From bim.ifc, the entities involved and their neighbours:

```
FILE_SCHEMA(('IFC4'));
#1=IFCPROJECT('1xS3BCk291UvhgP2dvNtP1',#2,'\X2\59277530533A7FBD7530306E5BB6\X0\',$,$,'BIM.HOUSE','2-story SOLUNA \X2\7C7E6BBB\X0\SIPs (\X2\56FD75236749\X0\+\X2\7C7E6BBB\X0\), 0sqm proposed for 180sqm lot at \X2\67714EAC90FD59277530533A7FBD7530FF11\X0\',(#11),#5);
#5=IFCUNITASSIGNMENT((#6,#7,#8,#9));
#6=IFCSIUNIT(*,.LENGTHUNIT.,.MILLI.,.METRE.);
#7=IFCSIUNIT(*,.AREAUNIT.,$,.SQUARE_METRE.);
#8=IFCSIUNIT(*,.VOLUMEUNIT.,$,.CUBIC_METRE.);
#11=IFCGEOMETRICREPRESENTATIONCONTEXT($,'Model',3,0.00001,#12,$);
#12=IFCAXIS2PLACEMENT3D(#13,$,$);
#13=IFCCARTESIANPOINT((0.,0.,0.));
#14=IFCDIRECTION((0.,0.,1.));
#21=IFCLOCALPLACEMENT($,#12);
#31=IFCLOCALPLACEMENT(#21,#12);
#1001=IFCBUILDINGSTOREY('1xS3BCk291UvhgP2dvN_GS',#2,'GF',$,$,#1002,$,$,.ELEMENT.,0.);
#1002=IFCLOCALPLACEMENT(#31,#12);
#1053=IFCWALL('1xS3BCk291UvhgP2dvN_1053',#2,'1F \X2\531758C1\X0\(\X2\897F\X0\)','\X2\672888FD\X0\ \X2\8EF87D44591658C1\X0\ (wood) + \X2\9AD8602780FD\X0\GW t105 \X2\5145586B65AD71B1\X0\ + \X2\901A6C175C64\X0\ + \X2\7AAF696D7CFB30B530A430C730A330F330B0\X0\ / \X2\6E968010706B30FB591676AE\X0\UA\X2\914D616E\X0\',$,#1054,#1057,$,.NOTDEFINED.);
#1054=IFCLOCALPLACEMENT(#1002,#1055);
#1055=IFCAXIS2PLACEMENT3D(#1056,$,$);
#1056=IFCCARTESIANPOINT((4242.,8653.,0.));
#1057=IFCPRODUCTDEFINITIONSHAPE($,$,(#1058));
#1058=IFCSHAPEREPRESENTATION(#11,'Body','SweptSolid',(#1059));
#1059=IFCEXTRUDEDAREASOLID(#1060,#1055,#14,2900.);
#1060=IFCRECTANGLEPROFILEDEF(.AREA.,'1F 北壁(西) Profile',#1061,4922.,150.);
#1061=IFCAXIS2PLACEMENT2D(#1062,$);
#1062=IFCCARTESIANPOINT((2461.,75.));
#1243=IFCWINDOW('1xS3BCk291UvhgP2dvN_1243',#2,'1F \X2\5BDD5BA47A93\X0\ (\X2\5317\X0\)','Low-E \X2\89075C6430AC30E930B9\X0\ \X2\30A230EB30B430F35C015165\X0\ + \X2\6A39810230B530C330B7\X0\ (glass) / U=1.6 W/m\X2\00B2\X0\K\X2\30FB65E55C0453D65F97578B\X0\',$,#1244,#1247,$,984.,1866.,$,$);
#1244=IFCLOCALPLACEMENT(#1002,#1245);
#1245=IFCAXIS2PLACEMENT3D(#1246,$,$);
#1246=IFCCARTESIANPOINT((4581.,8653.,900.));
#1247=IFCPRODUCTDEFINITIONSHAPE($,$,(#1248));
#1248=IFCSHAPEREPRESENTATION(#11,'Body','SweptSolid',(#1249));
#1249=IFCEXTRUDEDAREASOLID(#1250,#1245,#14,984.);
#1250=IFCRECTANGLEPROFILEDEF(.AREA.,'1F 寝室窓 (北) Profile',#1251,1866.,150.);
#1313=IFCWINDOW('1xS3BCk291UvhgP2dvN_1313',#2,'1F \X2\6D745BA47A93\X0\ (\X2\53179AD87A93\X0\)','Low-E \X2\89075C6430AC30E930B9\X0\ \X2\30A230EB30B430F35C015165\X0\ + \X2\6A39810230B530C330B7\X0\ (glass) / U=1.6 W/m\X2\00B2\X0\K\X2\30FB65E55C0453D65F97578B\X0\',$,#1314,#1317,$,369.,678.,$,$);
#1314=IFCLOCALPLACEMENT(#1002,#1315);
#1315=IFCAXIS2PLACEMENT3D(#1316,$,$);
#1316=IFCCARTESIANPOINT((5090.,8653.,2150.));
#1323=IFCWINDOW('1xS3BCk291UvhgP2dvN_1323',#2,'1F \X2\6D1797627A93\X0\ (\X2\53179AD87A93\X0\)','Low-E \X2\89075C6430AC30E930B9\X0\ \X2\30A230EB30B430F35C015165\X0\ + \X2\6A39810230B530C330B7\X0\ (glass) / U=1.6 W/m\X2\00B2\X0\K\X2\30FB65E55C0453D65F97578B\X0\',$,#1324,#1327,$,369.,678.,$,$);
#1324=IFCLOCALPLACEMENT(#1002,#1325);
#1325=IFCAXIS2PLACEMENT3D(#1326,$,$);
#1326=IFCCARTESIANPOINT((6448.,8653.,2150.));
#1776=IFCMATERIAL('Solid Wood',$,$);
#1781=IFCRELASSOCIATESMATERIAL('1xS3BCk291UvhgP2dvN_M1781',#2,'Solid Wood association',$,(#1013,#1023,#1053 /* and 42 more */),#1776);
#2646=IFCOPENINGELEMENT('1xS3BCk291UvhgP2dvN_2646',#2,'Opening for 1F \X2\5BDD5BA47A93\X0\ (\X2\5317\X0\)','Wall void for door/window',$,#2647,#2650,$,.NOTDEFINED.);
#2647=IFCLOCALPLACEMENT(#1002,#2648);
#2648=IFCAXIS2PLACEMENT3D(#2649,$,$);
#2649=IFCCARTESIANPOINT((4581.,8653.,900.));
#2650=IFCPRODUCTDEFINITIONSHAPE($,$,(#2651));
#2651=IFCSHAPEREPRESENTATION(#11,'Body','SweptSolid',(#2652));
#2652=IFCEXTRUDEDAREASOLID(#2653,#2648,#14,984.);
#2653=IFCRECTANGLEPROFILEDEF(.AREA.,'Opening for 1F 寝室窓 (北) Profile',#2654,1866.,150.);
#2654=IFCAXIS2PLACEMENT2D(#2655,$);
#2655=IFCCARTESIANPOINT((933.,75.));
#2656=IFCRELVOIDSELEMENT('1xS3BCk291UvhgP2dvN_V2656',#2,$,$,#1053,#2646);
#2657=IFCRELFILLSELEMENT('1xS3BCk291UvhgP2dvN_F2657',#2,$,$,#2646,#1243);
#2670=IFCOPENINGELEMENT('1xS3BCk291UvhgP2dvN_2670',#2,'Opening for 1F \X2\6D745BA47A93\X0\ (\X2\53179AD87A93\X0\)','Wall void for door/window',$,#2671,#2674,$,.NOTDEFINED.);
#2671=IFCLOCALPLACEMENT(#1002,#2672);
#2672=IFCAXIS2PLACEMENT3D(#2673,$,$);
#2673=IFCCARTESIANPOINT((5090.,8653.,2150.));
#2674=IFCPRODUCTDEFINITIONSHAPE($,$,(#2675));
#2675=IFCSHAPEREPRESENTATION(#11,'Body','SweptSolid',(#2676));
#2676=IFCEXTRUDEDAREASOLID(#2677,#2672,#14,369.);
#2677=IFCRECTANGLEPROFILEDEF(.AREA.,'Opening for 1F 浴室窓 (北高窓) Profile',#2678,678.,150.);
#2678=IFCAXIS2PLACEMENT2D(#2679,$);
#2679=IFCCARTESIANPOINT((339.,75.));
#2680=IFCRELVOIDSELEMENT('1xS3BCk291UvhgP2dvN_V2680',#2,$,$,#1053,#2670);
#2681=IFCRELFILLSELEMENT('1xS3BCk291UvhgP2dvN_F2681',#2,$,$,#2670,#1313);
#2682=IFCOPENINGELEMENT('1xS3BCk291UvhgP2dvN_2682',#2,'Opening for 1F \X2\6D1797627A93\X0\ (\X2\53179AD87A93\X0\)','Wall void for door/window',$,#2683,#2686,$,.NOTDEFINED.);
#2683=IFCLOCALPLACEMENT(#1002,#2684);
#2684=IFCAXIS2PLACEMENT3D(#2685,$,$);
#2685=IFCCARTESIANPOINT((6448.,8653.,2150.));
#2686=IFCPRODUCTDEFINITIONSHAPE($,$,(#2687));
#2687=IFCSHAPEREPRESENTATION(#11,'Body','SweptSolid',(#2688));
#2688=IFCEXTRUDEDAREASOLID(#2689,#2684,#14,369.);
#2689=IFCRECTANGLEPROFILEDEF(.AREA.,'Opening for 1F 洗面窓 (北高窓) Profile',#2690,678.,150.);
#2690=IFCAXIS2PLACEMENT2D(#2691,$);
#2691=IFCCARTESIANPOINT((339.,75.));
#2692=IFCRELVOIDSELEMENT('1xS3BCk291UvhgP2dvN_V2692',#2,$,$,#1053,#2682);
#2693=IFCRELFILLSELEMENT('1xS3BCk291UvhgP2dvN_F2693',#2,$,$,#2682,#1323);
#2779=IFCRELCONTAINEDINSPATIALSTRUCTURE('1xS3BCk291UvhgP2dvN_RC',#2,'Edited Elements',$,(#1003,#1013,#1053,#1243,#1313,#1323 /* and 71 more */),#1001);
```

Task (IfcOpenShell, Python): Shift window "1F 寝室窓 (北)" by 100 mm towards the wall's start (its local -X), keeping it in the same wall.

```python
import ifcopenshell
import ifcopenshell.api.geometry
import ifcopenshell.util.placement

model = ifcopenshell.open("bim.ifc")

window = model.by_id(1243)
opening = window.FillsVoids[0].RelatingOpeningElement
wall = opening.VoidsElements[0].RelatingBuildingElement

wall_matrix = ifcopenshell.util.placement.get_local_placement(wall.ObjectPlacement)
shift = wall_matrix[:3, 0] * -100.0
before = ifcopenshell.util.placement.get_local_placement(window.ObjectPlacement)[:3, 3].copy()

# The window is not placed relative to its opening, so move both.
for product in (opening, window):
    matrix = ifcopenshell.util.placement.get_local_placement(product.ObjectPlacement)
    matrix[:3, 3] += shift
    ifcopenshell.api.geometry.edit_object_placement(model, product=product, matrix=matrix, is_si=False)

after = ifcopenshell.util.placement.get_local_placement(window.ObjectPlacement)[:3, 3]
print("window moved by", (after - before).round(3) + 0.0)

model.write("bim_updated.ifc")
```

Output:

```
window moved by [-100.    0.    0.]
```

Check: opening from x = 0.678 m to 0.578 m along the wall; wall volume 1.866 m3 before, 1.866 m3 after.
